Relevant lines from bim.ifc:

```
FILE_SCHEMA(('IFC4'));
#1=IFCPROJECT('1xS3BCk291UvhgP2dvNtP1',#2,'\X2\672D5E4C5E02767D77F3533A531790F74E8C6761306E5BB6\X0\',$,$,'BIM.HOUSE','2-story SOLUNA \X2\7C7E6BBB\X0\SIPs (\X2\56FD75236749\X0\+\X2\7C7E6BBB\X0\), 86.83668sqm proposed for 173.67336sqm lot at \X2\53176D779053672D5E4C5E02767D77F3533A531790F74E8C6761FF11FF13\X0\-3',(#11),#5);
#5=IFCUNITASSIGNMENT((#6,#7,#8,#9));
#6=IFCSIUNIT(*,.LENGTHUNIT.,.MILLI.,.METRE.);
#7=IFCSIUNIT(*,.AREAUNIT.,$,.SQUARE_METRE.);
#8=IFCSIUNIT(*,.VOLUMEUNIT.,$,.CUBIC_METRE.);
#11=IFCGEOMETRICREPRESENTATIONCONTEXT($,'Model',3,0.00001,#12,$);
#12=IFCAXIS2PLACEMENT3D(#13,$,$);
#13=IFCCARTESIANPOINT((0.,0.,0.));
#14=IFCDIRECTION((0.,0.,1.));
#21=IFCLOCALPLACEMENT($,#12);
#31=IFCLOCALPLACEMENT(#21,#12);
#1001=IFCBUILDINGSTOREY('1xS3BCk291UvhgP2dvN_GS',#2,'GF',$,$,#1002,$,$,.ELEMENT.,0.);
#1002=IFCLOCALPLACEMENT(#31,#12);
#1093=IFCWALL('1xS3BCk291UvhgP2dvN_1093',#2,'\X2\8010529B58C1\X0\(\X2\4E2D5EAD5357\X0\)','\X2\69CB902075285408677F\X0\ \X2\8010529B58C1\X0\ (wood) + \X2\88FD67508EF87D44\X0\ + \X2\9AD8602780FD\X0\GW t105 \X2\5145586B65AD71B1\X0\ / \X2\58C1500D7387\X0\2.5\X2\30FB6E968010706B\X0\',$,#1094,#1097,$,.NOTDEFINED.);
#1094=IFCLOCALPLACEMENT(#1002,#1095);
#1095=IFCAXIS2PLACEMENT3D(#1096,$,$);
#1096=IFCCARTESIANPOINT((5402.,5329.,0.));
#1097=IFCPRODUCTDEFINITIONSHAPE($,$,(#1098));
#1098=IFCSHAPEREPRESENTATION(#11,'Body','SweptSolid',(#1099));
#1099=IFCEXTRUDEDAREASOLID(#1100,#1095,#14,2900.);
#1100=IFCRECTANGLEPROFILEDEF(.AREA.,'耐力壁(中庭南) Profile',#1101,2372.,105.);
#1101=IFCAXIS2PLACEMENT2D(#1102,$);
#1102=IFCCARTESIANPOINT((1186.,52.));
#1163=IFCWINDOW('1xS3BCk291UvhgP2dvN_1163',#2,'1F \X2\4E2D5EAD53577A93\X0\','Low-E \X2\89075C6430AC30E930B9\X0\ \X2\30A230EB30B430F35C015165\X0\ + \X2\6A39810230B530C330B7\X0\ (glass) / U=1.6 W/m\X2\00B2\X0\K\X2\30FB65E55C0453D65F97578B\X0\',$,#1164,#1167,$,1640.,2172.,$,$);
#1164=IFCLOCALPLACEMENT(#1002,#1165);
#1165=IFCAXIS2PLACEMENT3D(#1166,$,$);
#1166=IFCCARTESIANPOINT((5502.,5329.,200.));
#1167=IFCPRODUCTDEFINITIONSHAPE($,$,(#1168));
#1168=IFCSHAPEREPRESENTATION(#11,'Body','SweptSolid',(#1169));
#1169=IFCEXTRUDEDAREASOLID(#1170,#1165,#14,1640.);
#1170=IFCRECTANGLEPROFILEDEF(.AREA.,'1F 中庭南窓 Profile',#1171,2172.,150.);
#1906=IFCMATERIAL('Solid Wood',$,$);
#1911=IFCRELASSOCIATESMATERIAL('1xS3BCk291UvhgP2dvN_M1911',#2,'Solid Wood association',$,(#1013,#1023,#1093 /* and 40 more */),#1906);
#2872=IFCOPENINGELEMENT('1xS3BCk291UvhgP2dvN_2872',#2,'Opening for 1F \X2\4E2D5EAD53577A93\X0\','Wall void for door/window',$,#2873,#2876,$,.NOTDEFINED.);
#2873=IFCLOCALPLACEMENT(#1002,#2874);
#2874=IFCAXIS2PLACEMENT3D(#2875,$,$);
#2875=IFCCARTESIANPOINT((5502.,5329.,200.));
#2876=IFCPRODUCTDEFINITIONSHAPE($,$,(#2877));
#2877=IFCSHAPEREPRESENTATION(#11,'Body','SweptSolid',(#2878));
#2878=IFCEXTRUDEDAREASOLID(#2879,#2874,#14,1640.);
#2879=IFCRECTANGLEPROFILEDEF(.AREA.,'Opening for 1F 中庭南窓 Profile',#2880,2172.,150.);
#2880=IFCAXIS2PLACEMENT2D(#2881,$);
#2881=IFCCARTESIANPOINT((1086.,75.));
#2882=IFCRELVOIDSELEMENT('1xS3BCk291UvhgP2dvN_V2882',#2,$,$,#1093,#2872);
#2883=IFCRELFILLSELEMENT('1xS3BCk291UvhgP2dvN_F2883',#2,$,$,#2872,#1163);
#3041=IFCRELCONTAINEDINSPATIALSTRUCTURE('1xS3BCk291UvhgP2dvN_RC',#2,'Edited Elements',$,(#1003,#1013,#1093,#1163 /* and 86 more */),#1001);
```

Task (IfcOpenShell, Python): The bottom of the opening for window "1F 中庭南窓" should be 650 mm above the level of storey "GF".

```python
import numpy as np
import ifcopenshell
import ifcopenshell.api.geometry
import ifcopenshell.geom
import ifcopenshell.util.element
import ifcopenshell.util.placement
import ifcopenshell.util.shape
import ifcopenshell.util.unit

model = ifcopenshell.open("bim.ifc")
unit_scale = ifcopenshell.util.unit.calculate_unit_scale(model)

window = model.by_guid("1xS3BCk291UvhgP2dvN_1163")
opening = window.FillsVoids[0].RelatingOpeningElement
storey = ifcopenshell.util.element.get_container(window, ifc_class="IfcBuildingStorey")
level = ifcopenshell.util.placement.get_local_placement(storey.ObjectPlacement)[2, 3]

# The opening's origin need not be at the sill, so measure its lowest point.
shape = ifcopenshell.geom.create_shape(ifcopenshell.geom.settings(), opening)
bottom = ifcopenshell.util.shape.get_shape_bottom_elevation(shape, shape.geometry) / unit_scale
dz = level + 0.65 / unit_scale - bottom

shift = np.array([0.0, 0.0, dz])
# The window is not placed relative to its opening, so move both.
for product in (opening, window):
    matrix = ifcopenshell.util.placement.get_local_placement(product.ObjectPlacement)
    matrix[:3, 3] += shift
    ifcopenshell.api.geometry.edit_object_placement(model, product=product, matrix=matrix, is_si=False)

print(f"moved by {dz * unit_scale:+.3f} m")

model.write("bim_updated.ifc")
```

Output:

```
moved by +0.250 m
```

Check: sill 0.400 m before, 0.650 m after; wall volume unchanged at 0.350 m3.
